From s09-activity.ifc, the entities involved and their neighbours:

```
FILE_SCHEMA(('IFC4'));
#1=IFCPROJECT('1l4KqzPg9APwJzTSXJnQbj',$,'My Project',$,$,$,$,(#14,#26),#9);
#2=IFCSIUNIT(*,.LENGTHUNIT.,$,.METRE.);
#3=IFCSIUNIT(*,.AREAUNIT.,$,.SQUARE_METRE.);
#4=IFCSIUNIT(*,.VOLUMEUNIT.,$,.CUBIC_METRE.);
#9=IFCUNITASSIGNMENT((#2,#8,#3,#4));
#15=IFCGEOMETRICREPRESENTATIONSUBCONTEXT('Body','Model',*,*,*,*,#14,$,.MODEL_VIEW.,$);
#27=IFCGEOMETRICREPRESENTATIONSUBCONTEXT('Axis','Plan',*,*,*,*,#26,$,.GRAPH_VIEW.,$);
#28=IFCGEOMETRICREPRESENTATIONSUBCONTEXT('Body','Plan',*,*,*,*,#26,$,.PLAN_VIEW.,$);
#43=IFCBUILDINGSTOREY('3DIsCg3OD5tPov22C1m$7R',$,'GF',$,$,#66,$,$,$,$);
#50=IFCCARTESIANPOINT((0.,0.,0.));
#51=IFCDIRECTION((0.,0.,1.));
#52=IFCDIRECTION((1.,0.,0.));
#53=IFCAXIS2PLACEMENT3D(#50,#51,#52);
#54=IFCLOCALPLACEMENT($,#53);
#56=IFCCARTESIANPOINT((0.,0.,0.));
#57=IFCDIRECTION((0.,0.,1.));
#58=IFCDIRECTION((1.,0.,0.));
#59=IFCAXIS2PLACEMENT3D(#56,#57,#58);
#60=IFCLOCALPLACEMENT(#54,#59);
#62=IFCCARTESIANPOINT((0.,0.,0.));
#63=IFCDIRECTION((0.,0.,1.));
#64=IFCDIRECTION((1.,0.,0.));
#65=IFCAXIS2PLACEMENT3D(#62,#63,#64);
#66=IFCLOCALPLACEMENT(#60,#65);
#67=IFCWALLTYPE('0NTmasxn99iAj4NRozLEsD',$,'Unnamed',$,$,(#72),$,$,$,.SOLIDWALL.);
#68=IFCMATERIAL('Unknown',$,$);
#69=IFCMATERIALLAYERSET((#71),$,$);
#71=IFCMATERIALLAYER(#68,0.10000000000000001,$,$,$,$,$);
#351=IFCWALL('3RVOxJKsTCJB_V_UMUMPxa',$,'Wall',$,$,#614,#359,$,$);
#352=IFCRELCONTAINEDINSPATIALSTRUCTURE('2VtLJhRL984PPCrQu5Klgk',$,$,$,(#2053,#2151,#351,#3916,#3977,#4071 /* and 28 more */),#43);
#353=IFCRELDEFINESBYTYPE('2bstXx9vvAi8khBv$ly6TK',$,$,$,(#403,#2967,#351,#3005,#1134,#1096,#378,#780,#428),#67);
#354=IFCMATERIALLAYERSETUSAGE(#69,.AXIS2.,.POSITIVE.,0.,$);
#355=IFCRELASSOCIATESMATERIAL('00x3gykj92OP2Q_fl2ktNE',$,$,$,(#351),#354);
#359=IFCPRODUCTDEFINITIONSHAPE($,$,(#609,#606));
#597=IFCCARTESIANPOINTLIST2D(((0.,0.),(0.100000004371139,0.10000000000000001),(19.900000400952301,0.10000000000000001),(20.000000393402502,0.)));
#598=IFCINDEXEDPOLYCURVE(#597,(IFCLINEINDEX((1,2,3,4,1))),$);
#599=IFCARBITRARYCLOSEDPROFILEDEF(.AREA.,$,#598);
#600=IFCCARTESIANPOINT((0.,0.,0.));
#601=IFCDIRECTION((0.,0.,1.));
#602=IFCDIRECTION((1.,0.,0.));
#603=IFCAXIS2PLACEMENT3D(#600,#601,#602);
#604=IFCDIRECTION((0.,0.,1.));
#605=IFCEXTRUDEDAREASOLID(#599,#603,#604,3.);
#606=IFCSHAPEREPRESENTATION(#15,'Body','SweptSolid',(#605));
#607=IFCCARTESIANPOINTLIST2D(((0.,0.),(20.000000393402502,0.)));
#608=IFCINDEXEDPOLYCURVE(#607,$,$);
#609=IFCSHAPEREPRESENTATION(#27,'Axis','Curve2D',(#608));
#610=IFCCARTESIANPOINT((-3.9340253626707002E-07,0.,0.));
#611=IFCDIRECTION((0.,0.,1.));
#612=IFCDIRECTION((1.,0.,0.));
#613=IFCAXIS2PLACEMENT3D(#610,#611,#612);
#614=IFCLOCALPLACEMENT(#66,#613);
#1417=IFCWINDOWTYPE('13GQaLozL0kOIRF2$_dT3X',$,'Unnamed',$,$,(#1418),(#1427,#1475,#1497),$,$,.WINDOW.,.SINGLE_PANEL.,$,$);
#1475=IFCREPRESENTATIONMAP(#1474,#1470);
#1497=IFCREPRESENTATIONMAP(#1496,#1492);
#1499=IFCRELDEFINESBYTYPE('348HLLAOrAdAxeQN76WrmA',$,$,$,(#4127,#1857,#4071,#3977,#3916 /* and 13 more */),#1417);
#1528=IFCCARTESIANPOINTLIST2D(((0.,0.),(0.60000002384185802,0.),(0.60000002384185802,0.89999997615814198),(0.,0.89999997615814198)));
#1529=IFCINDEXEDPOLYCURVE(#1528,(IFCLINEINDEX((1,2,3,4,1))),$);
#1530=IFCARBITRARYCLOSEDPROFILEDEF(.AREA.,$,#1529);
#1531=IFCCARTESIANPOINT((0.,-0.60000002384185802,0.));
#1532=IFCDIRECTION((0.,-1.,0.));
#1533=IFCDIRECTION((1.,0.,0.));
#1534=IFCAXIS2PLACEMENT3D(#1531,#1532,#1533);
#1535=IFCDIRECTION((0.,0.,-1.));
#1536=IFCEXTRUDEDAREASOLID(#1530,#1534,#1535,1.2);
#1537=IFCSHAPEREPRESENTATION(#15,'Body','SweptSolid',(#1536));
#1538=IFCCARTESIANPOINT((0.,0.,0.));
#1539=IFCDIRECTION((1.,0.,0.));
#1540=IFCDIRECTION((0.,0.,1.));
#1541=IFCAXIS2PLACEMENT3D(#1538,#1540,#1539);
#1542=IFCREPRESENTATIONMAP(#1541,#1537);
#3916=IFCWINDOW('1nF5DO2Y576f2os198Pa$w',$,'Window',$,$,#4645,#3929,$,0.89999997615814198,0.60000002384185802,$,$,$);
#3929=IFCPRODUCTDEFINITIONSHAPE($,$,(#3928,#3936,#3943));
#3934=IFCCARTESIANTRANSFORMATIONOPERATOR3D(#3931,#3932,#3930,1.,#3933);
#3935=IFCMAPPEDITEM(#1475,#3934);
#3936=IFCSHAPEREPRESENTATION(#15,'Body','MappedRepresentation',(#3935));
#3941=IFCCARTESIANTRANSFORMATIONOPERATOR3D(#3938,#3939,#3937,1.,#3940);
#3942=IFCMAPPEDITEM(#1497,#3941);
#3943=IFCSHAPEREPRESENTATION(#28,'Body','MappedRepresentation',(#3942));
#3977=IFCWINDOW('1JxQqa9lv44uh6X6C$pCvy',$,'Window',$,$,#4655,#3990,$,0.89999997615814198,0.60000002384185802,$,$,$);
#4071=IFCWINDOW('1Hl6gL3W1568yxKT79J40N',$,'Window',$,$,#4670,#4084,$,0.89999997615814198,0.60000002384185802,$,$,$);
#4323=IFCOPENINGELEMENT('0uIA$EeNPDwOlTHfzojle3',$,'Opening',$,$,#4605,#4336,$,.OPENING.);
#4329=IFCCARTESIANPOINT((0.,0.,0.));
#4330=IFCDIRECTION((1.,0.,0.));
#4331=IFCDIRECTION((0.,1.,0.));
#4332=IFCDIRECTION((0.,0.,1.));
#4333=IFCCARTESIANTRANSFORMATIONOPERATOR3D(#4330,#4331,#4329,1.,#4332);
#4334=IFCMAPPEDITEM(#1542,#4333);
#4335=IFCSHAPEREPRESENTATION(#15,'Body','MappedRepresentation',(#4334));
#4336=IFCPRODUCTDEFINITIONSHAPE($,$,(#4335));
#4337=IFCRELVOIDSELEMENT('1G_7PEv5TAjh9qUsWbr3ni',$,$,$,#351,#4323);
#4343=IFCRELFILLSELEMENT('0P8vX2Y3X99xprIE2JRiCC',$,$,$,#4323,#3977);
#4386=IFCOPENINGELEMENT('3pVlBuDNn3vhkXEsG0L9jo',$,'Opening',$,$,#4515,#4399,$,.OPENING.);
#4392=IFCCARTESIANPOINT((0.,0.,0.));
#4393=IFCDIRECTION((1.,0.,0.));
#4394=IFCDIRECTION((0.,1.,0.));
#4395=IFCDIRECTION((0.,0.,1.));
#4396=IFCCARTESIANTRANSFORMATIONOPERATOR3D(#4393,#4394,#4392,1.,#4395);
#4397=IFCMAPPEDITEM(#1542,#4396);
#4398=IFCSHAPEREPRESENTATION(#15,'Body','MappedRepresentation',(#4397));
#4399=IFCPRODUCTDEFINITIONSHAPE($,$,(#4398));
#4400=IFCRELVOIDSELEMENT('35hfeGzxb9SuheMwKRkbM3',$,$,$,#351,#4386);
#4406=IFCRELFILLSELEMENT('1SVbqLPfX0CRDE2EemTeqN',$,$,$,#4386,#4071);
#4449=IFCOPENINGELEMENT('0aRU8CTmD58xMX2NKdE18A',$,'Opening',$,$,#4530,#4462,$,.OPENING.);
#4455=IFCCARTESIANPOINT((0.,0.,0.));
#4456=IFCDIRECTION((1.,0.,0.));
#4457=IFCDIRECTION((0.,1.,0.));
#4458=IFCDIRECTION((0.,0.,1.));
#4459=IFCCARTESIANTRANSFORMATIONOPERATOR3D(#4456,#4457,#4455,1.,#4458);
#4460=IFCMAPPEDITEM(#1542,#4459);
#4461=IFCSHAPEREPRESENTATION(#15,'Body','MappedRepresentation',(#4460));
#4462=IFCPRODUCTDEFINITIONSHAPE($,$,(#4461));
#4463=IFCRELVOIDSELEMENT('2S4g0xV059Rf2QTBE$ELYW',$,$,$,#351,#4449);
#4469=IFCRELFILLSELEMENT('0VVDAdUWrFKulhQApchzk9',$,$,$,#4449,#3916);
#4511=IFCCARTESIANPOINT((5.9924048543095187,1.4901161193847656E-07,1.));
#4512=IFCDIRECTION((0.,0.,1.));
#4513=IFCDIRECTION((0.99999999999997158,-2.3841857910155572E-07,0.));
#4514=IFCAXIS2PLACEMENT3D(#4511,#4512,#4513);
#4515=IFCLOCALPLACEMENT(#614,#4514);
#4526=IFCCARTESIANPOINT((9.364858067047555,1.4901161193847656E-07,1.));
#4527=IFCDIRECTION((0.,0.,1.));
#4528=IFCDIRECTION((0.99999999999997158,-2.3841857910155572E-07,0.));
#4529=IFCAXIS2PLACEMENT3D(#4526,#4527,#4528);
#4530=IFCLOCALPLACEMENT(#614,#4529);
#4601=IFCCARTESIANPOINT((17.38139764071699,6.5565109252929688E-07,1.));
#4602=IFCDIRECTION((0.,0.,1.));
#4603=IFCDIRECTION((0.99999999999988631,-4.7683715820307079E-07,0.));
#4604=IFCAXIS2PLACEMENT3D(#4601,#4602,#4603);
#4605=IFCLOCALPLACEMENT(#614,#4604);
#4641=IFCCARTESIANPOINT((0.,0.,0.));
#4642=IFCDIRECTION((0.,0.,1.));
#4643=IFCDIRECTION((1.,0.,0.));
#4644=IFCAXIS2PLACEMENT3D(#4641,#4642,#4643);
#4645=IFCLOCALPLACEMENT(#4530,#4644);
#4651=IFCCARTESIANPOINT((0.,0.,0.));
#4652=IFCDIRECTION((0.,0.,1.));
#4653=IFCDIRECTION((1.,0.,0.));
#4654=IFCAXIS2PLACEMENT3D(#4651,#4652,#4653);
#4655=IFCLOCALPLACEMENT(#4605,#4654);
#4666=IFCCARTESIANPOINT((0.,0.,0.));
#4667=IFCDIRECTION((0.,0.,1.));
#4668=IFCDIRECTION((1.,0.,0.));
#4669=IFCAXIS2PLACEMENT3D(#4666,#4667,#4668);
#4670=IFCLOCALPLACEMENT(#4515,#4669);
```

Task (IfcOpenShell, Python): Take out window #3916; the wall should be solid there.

```python
import ifcopenshell
import ifcopenshell.api.feature
import ifcopenshell.api.root
import ifcopenshell.geom
import ifcopenshell.util.shape

model = ifcopenshell.open("s09-activity.ifc")
settings = ifcopenshell.geom.settings()


def volume(element):
    """Net volume in cubic metres, openings subtracted."""
    shape = ifcopenshell.geom.create_shape(settings, element)
    return ifcopenshell.util.shape.get_volume(shape.geometry)


window = model.by_guid("1nF5DO2Y576f2os198Pa$w")
opening = window.FillsVoids[0].RelatingOpeningElement
wall = opening.VoidsElements[0].RelatingBuildingElement
before = volume(wall)

ifcopenshell.api.root.remove_product(model, product=window)
ifcopenshell.api.feature.remove_feature(model, feature=opening)

after = volume(wall)

print(f"wall volume {before:.3f} -> {after:.3f} m3")

model.write("s09-activity_v2.ifc")
```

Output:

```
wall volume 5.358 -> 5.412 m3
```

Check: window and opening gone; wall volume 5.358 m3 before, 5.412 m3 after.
